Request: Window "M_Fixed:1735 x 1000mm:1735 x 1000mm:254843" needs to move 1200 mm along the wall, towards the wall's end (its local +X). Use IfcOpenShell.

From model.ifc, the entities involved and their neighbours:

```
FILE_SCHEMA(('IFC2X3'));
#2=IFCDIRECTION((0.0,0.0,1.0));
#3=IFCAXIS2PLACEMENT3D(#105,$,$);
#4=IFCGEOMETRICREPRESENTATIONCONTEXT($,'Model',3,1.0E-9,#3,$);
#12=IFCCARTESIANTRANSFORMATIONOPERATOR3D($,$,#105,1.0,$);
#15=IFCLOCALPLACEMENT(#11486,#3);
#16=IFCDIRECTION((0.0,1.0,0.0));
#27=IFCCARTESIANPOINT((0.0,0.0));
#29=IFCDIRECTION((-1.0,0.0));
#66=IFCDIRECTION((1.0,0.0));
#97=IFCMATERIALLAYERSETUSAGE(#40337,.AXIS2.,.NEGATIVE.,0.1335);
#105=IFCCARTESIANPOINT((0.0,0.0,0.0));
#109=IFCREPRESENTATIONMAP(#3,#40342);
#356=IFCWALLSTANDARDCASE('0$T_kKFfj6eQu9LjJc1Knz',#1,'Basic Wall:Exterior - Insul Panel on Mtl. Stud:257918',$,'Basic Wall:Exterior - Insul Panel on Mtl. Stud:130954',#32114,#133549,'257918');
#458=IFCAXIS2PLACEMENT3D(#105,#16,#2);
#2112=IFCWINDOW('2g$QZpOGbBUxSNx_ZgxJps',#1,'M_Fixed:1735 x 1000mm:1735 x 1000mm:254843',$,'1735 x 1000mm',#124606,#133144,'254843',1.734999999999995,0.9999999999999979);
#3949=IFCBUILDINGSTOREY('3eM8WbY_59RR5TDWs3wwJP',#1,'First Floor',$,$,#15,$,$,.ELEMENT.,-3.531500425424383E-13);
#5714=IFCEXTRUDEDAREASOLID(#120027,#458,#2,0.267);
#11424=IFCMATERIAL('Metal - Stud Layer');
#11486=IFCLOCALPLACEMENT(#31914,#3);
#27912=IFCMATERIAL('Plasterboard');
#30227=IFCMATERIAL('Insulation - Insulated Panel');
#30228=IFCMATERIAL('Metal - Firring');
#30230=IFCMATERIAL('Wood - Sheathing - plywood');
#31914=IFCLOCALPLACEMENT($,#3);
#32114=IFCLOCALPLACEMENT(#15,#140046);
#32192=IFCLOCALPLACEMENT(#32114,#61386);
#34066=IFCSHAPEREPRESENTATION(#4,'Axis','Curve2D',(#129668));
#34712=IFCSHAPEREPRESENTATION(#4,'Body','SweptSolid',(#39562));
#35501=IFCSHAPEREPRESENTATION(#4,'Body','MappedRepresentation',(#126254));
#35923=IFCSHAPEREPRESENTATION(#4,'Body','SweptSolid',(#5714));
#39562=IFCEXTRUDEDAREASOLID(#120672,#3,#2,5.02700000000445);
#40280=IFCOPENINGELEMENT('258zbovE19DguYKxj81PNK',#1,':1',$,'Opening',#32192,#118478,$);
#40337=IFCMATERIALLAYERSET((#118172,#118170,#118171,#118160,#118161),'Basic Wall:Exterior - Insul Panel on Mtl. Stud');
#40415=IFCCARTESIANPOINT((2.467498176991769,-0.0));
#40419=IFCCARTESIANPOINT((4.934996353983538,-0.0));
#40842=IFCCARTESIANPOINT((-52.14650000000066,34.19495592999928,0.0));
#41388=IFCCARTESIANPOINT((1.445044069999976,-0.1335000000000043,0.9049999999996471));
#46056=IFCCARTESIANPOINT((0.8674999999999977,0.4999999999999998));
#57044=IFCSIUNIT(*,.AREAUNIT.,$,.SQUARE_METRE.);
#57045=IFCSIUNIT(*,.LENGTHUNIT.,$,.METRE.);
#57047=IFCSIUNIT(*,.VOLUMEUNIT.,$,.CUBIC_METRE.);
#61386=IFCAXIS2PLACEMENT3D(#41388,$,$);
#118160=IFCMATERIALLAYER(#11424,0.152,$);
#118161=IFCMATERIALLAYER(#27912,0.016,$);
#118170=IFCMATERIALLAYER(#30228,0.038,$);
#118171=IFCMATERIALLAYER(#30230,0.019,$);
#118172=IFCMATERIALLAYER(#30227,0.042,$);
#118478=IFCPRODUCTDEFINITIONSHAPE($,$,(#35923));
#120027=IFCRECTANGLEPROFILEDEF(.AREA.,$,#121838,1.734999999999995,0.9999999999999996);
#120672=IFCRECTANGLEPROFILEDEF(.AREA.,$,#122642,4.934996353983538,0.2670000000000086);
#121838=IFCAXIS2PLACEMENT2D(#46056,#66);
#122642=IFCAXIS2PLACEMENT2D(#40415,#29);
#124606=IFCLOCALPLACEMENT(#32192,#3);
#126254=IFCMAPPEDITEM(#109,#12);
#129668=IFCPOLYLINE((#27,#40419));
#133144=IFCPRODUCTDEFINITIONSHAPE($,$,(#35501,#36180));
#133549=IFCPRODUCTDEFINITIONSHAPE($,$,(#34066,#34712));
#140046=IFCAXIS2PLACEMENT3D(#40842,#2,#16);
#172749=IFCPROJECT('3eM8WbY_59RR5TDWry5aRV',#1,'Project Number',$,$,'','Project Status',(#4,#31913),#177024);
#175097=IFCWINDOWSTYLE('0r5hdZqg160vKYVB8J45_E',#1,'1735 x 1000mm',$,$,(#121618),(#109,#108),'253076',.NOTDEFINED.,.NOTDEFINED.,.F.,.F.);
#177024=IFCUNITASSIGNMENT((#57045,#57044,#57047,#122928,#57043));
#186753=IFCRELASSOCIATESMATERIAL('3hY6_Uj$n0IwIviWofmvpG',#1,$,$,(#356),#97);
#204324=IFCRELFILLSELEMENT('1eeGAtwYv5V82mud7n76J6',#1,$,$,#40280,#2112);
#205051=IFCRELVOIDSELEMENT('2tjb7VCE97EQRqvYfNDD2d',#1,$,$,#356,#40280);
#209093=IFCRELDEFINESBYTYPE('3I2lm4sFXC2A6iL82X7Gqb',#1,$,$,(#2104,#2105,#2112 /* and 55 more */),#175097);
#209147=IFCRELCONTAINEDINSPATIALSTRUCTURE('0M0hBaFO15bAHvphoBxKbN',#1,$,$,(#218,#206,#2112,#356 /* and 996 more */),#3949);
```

```python
import ifcopenshell
import ifcopenshell.api.geometry
import ifcopenshell.util.placement
import ifcopenshell.util.unit

model = ifcopenshell.open("model.ifc")
unit_scale = ifcopenshell.util.unit.calculate_unit_scale(model)

window = model.by_guid("2g$QZpOGbBUxSNx_ZgxJps")
opening = window.FillsVoids[0].RelatingOpeningElement
wall = opening.VoidsElements[0].RelatingBuildingElement

wall_matrix = ifcopenshell.util.placement.get_local_placement(wall.ObjectPlacement)
shift = wall_matrix[:3, 0] * 1.2 / unit_scale
before = ifcopenshell.util.placement.get_local_placement(window.ObjectPlacement)[:3, 3].copy()

# The window is placed relative to its opening, so it follows when the opening moves.
matrix = ifcopenshell.util.placement.get_local_placement(opening.ObjectPlacement)
matrix[:3, 3] += shift
ifcopenshell.api.geometry.edit_object_placement(
    model, product=opening, matrix=matrix, is_si=False, should_transform_children=True
)

after = ifcopenshell.util.placement.get_local_placement(window.ObjectPlacement)[:3, 3]
print("window moved by", (after - before).round(3) + 0.0)

model.write("model_rev.ifc")
```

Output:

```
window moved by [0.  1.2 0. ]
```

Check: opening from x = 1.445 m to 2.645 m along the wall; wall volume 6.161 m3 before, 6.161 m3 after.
